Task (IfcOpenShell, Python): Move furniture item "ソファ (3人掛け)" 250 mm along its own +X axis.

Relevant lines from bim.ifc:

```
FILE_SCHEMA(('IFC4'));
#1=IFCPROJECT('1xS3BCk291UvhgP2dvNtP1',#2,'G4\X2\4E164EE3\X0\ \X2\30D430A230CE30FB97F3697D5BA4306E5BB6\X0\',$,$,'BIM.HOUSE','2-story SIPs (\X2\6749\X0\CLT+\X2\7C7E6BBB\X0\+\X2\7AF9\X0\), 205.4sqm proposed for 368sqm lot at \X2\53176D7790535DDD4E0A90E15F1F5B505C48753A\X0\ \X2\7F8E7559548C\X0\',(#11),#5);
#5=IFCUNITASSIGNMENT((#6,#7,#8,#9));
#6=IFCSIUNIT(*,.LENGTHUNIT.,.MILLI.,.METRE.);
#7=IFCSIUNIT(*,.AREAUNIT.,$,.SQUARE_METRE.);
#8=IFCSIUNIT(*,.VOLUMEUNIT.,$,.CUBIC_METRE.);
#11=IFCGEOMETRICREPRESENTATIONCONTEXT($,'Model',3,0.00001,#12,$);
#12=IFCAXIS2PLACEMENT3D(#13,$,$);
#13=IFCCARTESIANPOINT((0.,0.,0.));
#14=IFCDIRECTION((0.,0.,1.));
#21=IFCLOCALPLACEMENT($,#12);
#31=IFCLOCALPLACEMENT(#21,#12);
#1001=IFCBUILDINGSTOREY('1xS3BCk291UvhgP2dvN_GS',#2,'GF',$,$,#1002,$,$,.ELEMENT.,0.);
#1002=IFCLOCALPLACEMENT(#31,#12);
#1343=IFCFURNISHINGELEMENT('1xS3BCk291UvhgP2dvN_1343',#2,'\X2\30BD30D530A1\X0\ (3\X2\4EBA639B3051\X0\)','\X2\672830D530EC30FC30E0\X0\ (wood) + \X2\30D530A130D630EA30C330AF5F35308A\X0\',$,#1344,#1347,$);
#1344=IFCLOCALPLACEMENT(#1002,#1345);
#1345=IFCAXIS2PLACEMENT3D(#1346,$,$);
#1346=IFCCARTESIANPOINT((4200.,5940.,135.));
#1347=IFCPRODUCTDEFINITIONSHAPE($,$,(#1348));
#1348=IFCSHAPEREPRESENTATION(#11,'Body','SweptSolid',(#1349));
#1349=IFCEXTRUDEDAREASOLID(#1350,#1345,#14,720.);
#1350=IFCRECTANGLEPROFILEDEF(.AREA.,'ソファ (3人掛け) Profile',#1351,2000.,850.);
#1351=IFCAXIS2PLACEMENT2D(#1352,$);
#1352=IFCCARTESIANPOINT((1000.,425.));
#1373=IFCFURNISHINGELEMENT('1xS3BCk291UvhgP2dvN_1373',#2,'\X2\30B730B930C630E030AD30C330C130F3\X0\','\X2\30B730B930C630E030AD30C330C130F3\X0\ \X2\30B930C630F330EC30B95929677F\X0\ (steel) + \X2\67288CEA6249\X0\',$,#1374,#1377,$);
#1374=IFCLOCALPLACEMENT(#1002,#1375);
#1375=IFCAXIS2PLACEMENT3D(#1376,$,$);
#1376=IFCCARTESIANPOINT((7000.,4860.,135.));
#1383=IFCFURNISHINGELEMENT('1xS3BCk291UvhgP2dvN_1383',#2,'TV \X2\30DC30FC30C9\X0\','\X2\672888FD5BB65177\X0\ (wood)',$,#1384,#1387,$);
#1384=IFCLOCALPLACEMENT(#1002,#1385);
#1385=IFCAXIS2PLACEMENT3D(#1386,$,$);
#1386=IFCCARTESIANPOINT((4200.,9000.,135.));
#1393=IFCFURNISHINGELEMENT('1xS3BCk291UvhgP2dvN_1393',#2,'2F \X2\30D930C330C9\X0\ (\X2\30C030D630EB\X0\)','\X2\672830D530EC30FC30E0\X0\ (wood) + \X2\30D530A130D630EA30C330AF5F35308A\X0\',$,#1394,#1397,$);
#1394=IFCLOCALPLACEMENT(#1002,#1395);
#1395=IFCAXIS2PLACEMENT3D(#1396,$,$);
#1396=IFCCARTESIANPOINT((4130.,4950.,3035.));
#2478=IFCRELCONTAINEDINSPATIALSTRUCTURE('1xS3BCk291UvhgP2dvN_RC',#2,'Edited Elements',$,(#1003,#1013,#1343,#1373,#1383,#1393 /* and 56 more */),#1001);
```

```python
import ifcopenshell
import ifcopenshell.api.geometry
import ifcopenshell.util.placement
import ifcopenshell.util.unit

model = ifcopenshell.open("bim.ifc")
unit_scale = ifcopenshell.util.unit.calculate_unit_scale(model)

item = model.by_guid("1xS3BCk291UvhgP2dvN_1343")
matrix = ifcopenshell.util.placement.get_local_placement(item.ObjectPlacement)
matrix[:3, 3] += matrix[:3, 0] * 0.25 / unit_scale
ifcopenshell.api.geometry.edit_object_placement(model, product=item, matrix=matrix, is_si=False)

print(ifcopenshell.util.placement.get_local_placement(item.ObjectPlacement).round(3) + 0.0)

model.write("bim_updated.ifc")
```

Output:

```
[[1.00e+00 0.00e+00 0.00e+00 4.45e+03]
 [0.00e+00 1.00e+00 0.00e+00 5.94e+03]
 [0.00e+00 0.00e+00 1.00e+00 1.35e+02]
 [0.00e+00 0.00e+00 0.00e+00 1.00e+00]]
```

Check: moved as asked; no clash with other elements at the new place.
